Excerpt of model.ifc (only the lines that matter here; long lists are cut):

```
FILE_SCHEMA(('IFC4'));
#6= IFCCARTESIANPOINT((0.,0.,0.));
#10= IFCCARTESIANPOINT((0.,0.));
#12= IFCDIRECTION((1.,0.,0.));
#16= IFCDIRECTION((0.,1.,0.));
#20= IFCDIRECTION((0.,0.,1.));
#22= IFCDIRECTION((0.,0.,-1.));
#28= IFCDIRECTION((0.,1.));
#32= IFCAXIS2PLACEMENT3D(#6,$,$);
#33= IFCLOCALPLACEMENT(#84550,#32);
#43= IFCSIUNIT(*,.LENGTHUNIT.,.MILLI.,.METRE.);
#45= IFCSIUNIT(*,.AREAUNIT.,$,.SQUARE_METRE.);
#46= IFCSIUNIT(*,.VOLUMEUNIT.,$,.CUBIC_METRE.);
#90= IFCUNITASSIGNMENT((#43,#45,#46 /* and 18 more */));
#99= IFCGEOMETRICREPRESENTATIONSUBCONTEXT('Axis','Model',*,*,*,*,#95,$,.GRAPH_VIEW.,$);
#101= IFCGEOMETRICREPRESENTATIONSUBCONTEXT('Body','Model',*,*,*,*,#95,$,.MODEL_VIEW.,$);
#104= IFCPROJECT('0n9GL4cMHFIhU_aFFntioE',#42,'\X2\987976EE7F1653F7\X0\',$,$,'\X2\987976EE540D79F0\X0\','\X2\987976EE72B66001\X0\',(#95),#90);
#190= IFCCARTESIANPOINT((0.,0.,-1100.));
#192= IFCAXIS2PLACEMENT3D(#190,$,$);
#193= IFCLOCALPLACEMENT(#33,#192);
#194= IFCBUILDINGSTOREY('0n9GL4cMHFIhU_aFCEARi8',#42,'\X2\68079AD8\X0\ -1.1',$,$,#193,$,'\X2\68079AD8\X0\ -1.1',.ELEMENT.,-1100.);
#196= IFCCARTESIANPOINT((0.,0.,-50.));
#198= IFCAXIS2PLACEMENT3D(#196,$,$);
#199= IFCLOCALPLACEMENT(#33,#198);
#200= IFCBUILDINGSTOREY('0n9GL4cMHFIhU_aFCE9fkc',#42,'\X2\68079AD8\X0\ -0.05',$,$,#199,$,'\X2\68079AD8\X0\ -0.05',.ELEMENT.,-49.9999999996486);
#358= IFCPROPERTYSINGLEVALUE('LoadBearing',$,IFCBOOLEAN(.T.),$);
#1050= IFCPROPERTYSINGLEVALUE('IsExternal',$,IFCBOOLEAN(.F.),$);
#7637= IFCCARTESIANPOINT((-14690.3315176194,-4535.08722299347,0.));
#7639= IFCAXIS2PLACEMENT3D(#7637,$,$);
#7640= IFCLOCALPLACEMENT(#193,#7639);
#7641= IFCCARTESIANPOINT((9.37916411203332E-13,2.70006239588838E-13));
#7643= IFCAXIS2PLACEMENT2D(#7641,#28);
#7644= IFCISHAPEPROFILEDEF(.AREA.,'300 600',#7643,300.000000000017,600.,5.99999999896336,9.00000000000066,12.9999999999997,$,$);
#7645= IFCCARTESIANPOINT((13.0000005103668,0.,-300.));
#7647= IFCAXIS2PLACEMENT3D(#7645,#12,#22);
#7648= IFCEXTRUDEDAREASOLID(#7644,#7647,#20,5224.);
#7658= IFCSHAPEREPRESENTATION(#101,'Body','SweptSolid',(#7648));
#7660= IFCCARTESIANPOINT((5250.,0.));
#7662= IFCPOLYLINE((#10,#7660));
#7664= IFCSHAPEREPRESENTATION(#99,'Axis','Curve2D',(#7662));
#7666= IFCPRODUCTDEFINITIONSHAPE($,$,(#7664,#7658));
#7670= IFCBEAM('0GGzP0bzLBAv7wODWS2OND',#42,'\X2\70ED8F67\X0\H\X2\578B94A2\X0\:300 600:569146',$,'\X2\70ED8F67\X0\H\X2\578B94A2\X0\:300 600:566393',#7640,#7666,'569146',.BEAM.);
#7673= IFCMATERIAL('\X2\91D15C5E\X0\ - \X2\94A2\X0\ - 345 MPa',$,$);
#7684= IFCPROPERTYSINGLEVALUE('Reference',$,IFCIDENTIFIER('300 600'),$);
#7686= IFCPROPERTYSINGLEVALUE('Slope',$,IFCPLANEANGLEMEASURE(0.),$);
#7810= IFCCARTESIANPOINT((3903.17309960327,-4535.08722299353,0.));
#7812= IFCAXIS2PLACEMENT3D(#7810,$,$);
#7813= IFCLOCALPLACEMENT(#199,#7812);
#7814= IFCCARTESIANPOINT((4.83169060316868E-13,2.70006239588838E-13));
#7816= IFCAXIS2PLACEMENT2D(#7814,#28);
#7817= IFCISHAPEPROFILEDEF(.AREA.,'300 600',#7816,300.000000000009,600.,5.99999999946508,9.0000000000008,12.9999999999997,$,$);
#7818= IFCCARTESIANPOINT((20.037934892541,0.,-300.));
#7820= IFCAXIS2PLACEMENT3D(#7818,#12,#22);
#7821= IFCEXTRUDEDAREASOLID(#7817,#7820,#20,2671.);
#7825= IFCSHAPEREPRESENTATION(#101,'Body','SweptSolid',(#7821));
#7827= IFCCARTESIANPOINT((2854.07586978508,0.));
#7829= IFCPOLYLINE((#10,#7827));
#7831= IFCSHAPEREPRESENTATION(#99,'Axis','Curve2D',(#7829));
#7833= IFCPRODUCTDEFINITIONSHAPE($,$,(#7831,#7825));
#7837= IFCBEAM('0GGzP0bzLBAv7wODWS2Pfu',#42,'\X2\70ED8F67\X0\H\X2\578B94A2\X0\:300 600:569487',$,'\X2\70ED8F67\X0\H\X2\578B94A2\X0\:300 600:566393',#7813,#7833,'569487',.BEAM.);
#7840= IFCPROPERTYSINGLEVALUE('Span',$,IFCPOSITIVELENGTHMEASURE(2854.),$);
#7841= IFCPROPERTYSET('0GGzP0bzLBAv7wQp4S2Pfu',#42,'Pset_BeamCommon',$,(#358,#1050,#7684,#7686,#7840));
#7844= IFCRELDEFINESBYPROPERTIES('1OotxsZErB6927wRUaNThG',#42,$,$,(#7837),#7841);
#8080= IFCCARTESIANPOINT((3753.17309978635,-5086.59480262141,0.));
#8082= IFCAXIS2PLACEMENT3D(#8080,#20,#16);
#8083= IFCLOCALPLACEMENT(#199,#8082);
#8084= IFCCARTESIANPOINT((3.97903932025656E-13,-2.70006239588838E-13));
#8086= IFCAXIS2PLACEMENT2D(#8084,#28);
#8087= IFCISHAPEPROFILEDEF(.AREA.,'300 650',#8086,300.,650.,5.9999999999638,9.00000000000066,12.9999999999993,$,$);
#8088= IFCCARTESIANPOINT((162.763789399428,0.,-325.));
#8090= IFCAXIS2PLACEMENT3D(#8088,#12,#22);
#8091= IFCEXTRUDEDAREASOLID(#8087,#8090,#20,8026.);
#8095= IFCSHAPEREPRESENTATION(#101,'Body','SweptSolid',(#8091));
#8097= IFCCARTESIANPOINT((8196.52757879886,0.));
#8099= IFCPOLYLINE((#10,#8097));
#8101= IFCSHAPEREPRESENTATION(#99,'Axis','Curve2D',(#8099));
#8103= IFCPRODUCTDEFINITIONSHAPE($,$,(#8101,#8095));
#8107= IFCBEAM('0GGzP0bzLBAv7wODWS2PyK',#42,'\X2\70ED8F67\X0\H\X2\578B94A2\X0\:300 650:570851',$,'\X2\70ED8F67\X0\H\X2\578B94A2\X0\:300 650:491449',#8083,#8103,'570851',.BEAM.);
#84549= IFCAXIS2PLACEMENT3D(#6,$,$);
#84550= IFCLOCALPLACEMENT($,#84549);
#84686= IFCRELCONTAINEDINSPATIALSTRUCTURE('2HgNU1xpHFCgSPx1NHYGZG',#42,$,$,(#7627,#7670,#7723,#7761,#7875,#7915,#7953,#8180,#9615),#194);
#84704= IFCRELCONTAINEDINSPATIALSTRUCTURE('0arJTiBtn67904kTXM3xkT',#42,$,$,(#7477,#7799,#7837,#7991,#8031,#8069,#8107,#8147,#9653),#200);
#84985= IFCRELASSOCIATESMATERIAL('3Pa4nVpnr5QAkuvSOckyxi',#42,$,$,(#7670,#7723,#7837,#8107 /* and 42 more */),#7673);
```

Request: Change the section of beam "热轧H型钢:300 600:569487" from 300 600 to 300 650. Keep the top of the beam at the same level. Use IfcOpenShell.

```python
import ifcopenshell
import ifcopenshell.api.pset
import ifcopenshell.util.element
import ifcopenshell.util.representation

model = ifcopenshell.open("model.ifc")

member = model.by_id(7837)
source = next(p for p in model.by_type("IfcIShapeProfileDef") if p.ProfileName == "300 650")

body = ifcopenshell.util.representation.get_representation(member, "Model", "Body")
solid = body.Items[0]
old_profile = solid.SweptArea

# Copy the section's sizes but keep this member's own profile position.
profile = ifcopenshell.util.element.copy(model, source)
# Profiles are centred, so shift by half the change in depth to hold the top.
shift = (old_profile.OverallDepth - profile.OverallDepth) / 2
x, y = old_profile.Position.Location.Coordinates
up = (-1.0, 0.0)  # upwards, in the solid's own plane
location = model.createIfcCartesianPoint((x + up[0] * shift, y + up[1] * shift))
profile.Position = model.createIfcAxis2Placement2D(location, old_profile.Position.RefDirection)
solid.SweptArea = profile
if not model.get_total_inverses(old_profile):
    ifcopenshell.util.element.remove_deep2(model, old_profile)
member.Name = member.Name.replace("300 600", "300 650")
member.ObjectType = member.ObjectType.replace("300 600", "300 650")
pset = model.by_id(ifcopenshell.util.element.get_pset(member, "Pset_BeamCommon", should_inherit=False)["id"])
ifcopenshell.api.pset.edit_pset(model, pset=pset, properties={"Reference": "300 650"})

print(solid.SweptArea)

model.write("model_updated.ifc")
```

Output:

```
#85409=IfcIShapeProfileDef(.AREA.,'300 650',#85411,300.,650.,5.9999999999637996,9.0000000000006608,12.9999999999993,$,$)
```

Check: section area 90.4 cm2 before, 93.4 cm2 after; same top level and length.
